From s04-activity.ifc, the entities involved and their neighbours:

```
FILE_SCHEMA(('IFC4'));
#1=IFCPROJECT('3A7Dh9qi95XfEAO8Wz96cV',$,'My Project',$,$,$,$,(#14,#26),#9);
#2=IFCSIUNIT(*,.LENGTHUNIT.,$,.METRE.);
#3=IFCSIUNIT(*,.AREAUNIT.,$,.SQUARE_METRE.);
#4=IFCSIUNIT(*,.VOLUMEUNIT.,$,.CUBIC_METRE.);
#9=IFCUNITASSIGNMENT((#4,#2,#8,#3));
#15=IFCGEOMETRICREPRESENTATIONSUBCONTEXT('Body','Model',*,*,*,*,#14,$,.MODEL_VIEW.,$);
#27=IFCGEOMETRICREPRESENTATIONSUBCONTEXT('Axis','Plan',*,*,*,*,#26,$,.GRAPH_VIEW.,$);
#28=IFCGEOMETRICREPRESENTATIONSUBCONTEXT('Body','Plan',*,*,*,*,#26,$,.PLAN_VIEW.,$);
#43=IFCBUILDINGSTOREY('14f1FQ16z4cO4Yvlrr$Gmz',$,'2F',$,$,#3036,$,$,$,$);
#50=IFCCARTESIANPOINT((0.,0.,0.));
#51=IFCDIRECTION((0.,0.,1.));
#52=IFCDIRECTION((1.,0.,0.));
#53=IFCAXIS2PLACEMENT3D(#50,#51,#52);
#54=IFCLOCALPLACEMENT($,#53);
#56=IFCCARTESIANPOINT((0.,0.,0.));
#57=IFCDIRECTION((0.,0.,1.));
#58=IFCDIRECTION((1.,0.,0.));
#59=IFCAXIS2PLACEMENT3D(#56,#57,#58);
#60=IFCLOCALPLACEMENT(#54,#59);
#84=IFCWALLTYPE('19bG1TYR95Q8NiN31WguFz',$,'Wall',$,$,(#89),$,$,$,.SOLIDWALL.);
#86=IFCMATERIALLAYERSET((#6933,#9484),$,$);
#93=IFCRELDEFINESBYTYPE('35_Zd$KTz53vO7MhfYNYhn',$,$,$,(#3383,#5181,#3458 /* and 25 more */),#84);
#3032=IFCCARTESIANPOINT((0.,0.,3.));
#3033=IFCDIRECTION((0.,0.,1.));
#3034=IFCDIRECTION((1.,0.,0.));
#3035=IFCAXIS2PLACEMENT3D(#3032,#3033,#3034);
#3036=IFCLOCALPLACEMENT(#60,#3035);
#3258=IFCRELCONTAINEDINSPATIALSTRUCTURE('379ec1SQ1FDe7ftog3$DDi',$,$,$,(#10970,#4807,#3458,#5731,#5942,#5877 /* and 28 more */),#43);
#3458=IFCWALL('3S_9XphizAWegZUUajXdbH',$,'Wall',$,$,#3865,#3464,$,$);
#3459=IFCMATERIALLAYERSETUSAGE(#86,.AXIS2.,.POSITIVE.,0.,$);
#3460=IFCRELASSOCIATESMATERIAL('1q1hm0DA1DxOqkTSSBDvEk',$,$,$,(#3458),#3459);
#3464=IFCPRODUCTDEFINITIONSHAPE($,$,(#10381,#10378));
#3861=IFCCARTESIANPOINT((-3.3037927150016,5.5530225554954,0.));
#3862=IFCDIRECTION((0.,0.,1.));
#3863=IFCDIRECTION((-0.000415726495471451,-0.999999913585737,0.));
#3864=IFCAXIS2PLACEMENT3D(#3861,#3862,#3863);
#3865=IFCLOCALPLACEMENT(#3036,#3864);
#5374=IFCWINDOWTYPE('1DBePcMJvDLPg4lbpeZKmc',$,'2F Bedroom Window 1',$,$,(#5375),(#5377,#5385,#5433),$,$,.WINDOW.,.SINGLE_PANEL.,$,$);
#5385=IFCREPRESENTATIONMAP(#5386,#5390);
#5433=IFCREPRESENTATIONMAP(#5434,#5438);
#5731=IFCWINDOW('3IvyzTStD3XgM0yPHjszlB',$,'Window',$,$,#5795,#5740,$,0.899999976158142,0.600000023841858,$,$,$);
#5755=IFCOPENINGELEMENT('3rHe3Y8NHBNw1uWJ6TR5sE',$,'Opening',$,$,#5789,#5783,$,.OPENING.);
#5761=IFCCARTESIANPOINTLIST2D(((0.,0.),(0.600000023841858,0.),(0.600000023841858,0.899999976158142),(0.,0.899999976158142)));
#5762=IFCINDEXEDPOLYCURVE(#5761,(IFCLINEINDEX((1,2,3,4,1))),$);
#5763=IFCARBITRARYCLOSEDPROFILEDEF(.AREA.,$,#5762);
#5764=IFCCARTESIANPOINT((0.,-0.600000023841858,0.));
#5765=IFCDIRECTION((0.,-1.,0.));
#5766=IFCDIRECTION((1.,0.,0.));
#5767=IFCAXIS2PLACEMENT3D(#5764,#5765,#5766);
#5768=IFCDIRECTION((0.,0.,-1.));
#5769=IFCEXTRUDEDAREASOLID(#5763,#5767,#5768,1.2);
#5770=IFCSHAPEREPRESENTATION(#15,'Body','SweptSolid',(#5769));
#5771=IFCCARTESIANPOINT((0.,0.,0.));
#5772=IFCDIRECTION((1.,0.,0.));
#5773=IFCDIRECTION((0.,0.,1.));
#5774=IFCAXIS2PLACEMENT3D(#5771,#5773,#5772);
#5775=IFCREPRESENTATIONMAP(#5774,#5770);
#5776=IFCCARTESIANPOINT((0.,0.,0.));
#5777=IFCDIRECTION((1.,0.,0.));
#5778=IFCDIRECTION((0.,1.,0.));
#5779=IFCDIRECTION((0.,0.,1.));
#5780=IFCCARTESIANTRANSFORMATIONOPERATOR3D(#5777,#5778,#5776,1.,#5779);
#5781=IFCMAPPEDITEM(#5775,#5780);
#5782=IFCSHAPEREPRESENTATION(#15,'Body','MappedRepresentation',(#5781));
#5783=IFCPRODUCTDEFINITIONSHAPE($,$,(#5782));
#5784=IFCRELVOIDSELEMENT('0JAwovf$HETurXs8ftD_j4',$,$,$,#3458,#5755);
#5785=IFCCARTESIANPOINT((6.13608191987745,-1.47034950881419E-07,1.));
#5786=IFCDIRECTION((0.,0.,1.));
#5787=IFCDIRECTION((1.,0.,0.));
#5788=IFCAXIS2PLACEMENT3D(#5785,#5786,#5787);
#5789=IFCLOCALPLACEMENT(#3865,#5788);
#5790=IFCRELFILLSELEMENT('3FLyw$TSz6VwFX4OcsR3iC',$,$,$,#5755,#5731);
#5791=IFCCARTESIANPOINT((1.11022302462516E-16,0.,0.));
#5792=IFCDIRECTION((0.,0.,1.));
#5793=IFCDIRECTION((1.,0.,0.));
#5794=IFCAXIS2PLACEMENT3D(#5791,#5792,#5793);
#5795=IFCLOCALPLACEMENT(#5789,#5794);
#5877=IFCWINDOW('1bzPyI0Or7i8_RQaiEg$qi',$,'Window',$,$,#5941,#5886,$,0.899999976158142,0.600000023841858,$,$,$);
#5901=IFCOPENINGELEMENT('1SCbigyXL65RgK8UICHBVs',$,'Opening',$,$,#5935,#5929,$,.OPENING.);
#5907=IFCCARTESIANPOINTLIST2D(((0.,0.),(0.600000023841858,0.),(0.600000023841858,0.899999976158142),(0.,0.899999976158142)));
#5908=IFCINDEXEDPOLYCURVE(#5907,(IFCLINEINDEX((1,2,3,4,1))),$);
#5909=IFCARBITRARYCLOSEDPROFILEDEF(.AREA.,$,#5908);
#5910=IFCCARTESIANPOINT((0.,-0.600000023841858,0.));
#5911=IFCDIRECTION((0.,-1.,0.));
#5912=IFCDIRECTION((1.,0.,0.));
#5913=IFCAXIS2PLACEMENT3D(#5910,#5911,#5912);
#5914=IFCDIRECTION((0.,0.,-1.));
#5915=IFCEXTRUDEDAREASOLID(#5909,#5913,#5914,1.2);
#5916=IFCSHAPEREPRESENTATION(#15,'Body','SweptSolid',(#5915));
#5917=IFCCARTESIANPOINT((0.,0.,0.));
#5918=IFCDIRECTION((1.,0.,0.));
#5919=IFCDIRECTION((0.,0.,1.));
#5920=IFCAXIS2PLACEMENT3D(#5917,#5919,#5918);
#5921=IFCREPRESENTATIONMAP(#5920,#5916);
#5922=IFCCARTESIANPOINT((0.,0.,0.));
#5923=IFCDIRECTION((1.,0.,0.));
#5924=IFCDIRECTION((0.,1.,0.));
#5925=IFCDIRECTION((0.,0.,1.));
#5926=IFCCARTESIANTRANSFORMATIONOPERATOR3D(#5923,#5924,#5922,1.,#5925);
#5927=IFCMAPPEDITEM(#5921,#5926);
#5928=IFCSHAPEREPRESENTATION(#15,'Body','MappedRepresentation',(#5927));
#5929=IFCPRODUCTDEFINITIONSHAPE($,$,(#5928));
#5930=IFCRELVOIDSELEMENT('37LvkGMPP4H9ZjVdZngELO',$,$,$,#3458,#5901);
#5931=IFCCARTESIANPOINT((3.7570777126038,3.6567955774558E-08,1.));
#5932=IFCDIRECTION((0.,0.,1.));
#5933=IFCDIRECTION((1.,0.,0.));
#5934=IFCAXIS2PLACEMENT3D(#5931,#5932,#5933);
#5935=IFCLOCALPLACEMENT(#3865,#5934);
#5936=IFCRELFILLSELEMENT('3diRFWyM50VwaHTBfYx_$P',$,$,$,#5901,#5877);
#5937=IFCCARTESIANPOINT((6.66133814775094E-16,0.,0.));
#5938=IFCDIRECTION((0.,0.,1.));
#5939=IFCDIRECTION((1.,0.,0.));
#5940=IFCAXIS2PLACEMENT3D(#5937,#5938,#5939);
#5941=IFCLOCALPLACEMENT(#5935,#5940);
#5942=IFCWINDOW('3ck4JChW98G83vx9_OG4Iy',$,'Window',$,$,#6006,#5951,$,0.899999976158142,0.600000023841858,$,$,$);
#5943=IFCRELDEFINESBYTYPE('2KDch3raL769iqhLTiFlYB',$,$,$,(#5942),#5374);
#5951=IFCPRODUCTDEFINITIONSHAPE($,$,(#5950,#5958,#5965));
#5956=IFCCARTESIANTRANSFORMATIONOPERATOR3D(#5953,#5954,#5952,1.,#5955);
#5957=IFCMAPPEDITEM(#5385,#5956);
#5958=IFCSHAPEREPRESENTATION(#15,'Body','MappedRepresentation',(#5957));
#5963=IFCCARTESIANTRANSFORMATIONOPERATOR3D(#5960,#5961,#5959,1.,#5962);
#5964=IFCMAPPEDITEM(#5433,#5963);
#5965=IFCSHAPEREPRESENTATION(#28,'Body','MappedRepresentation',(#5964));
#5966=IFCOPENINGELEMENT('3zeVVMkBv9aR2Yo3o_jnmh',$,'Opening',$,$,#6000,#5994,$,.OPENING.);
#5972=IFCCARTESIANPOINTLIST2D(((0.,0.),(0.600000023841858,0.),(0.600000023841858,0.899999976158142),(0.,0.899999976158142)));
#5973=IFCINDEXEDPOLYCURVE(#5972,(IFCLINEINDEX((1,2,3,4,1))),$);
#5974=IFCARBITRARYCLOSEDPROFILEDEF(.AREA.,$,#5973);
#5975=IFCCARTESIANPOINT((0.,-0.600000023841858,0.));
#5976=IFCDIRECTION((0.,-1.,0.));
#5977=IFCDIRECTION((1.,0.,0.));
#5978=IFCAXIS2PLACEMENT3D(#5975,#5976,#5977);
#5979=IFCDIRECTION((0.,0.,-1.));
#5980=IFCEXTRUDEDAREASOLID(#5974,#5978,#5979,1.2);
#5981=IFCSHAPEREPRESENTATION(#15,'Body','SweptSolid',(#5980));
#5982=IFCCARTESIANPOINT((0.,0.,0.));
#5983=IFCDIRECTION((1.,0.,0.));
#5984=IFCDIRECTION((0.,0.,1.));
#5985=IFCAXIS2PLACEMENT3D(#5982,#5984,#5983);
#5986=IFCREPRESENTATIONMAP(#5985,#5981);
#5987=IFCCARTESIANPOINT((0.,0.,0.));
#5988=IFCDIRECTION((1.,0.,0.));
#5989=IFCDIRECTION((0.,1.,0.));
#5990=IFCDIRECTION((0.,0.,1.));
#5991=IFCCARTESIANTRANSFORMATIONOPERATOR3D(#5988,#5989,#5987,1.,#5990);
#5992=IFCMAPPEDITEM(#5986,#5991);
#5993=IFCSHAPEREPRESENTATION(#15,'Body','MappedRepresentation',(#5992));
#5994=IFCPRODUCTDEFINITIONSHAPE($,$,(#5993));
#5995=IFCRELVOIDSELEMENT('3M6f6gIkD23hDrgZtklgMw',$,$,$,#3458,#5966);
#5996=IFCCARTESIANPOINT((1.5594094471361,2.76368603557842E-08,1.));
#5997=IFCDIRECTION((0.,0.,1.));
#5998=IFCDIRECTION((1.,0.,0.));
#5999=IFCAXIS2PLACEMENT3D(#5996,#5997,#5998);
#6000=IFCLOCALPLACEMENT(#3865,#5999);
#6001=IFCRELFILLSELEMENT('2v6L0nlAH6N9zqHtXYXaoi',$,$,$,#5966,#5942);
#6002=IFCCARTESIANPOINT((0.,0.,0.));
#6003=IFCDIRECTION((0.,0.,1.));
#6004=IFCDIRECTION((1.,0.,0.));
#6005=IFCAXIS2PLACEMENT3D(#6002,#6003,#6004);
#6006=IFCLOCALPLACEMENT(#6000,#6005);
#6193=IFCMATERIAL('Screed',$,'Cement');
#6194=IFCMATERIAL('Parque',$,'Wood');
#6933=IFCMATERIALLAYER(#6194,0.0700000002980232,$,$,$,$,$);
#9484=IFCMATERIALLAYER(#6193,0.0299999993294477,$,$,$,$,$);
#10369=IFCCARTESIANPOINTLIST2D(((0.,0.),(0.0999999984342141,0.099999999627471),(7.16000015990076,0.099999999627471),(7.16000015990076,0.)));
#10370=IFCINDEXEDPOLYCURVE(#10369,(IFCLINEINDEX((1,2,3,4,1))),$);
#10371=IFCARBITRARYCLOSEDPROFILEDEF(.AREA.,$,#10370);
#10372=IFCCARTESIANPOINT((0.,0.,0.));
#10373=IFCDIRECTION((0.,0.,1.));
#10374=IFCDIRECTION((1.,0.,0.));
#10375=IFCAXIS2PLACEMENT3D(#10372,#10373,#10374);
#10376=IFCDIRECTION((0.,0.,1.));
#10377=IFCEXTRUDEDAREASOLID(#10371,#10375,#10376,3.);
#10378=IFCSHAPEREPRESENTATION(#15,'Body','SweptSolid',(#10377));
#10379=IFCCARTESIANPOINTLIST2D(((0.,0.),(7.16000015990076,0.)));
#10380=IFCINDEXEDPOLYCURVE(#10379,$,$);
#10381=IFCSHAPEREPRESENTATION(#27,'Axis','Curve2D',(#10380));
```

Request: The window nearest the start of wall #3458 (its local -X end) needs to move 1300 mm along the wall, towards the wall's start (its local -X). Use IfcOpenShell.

```python
import ifcopenshell
import ifcopenshell.api.geometry
import ifcopenshell.util.placement

model = ifcopenshell.open("s04-activity.ifc")

window = model.by_guid("3ck4JChW98G83vx9_OG4Iy")
opening = window.FillsVoids[0].RelatingOpeningElement
wall = opening.VoidsElements[0].RelatingBuildingElement

wall_matrix = ifcopenshell.util.placement.get_local_placement(wall.ObjectPlacement)
shift = wall_matrix[:3, 0] * -1.3
before = ifcopenshell.util.placement.get_local_placement(window.ObjectPlacement)[:3, 3].copy()

# The window is placed relative to its opening, so it follows when the opening moves.
matrix = ifcopenshell.util.placement.get_local_placement(opening.ObjectPlacement)
matrix[:3, 3] += shift
ifcopenshell.api.geometry.edit_object_placement(
    model, product=opening, matrix=matrix, is_si=False, should_transform_children=True
)

after = ifcopenshell.util.placement.get_local_placement(window.ObjectPlacement)[:3, 3]
print("window moved by", (after - before).round(3) + 0.0)

model.write("s04-activity-out.ifc")
```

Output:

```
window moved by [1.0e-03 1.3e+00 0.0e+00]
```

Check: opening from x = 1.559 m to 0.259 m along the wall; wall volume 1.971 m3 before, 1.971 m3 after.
